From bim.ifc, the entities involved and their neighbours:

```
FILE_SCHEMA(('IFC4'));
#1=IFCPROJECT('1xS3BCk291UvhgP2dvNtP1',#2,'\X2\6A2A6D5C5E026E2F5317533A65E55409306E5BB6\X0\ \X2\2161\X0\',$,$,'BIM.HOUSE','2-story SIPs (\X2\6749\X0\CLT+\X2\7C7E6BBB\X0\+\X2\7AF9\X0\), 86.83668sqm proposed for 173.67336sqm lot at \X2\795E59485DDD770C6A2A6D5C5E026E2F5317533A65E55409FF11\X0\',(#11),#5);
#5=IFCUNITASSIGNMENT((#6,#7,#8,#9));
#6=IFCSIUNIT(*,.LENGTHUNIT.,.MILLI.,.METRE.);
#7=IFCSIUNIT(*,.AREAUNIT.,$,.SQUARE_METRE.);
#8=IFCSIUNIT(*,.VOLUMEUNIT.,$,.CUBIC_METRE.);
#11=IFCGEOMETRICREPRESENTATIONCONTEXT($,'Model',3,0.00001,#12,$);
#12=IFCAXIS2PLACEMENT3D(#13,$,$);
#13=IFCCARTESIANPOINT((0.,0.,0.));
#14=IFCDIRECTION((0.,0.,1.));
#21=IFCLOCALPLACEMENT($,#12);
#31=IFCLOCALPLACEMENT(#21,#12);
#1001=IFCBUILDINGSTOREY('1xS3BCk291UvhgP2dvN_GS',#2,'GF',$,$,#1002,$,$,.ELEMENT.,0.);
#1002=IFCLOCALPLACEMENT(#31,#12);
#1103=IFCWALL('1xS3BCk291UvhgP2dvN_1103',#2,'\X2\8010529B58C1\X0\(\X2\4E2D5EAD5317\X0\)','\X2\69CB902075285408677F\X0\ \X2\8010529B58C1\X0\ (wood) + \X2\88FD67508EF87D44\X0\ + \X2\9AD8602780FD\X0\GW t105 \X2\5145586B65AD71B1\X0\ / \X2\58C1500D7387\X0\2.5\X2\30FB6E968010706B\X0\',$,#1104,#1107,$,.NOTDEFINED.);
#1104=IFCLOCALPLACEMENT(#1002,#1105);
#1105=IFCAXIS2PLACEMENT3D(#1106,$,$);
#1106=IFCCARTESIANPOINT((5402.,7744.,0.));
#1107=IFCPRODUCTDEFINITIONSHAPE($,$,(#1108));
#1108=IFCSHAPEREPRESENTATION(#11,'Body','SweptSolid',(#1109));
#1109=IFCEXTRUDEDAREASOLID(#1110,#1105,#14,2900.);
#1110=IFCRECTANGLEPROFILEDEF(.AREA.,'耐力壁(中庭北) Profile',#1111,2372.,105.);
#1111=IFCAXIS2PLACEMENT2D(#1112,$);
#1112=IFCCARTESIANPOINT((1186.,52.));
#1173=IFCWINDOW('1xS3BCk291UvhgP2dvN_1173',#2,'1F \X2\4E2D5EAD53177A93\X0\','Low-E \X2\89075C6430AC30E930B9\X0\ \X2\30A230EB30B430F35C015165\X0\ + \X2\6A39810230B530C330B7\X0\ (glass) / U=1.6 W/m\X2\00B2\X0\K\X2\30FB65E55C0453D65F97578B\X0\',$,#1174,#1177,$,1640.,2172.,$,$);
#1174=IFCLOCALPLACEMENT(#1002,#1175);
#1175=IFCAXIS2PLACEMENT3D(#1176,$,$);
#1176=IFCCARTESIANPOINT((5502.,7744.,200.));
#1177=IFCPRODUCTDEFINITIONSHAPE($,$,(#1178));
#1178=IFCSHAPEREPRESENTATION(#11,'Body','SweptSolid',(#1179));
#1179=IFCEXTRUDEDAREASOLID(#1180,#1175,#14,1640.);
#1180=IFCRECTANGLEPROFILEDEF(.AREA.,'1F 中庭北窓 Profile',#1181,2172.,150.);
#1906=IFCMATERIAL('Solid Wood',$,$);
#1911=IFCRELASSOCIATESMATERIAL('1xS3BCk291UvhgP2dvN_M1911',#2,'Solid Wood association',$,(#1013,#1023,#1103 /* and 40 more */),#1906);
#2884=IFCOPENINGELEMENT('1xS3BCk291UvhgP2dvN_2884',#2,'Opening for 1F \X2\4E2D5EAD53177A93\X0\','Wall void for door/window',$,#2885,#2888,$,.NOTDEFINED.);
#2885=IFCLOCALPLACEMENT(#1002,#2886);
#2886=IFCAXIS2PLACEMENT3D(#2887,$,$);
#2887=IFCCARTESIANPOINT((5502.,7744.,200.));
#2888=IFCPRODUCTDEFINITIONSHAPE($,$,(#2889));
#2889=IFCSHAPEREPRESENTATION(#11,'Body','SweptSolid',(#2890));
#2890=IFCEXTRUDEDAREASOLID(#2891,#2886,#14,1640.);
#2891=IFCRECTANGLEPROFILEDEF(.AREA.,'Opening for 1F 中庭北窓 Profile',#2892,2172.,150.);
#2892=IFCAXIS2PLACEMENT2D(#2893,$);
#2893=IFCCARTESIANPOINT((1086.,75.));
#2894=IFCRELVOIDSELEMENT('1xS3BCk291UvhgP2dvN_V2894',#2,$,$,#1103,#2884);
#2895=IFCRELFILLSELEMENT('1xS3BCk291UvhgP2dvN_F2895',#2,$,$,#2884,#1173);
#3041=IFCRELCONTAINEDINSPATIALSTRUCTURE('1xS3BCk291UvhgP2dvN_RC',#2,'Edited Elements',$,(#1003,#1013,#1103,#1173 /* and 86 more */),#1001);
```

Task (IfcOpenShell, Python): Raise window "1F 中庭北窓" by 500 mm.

```python
import numpy as np
import ifcopenshell
import ifcopenshell.api.geometry
import ifcopenshell.util.placement
import ifcopenshell.util.unit

model = ifcopenshell.open("bim.ifc")
unit_scale = ifcopenshell.util.unit.calculate_unit_scale(model)

window = model.by_guid("1xS3BCk291UvhgP2dvN_1173")
opening = window.FillsVoids[0].RelatingOpeningElement
dz = 0.5 / unit_scale

shift = np.array([0.0, 0.0, dz])
# The window is not placed relative to its opening, so move both.
for product in (opening, window):
    matrix = ifcopenshell.util.placement.get_local_placement(product.ObjectPlacement)
    matrix[:3, 3] += shift
    ifcopenshell.api.geometry.edit_object_placement(model, product=product, matrix=matrix, is_si=False)

print(f"moved by {dz * unit_scale:+.3f} m")

model.write("bim_edited.ifc")
```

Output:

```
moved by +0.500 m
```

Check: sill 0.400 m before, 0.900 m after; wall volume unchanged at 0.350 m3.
